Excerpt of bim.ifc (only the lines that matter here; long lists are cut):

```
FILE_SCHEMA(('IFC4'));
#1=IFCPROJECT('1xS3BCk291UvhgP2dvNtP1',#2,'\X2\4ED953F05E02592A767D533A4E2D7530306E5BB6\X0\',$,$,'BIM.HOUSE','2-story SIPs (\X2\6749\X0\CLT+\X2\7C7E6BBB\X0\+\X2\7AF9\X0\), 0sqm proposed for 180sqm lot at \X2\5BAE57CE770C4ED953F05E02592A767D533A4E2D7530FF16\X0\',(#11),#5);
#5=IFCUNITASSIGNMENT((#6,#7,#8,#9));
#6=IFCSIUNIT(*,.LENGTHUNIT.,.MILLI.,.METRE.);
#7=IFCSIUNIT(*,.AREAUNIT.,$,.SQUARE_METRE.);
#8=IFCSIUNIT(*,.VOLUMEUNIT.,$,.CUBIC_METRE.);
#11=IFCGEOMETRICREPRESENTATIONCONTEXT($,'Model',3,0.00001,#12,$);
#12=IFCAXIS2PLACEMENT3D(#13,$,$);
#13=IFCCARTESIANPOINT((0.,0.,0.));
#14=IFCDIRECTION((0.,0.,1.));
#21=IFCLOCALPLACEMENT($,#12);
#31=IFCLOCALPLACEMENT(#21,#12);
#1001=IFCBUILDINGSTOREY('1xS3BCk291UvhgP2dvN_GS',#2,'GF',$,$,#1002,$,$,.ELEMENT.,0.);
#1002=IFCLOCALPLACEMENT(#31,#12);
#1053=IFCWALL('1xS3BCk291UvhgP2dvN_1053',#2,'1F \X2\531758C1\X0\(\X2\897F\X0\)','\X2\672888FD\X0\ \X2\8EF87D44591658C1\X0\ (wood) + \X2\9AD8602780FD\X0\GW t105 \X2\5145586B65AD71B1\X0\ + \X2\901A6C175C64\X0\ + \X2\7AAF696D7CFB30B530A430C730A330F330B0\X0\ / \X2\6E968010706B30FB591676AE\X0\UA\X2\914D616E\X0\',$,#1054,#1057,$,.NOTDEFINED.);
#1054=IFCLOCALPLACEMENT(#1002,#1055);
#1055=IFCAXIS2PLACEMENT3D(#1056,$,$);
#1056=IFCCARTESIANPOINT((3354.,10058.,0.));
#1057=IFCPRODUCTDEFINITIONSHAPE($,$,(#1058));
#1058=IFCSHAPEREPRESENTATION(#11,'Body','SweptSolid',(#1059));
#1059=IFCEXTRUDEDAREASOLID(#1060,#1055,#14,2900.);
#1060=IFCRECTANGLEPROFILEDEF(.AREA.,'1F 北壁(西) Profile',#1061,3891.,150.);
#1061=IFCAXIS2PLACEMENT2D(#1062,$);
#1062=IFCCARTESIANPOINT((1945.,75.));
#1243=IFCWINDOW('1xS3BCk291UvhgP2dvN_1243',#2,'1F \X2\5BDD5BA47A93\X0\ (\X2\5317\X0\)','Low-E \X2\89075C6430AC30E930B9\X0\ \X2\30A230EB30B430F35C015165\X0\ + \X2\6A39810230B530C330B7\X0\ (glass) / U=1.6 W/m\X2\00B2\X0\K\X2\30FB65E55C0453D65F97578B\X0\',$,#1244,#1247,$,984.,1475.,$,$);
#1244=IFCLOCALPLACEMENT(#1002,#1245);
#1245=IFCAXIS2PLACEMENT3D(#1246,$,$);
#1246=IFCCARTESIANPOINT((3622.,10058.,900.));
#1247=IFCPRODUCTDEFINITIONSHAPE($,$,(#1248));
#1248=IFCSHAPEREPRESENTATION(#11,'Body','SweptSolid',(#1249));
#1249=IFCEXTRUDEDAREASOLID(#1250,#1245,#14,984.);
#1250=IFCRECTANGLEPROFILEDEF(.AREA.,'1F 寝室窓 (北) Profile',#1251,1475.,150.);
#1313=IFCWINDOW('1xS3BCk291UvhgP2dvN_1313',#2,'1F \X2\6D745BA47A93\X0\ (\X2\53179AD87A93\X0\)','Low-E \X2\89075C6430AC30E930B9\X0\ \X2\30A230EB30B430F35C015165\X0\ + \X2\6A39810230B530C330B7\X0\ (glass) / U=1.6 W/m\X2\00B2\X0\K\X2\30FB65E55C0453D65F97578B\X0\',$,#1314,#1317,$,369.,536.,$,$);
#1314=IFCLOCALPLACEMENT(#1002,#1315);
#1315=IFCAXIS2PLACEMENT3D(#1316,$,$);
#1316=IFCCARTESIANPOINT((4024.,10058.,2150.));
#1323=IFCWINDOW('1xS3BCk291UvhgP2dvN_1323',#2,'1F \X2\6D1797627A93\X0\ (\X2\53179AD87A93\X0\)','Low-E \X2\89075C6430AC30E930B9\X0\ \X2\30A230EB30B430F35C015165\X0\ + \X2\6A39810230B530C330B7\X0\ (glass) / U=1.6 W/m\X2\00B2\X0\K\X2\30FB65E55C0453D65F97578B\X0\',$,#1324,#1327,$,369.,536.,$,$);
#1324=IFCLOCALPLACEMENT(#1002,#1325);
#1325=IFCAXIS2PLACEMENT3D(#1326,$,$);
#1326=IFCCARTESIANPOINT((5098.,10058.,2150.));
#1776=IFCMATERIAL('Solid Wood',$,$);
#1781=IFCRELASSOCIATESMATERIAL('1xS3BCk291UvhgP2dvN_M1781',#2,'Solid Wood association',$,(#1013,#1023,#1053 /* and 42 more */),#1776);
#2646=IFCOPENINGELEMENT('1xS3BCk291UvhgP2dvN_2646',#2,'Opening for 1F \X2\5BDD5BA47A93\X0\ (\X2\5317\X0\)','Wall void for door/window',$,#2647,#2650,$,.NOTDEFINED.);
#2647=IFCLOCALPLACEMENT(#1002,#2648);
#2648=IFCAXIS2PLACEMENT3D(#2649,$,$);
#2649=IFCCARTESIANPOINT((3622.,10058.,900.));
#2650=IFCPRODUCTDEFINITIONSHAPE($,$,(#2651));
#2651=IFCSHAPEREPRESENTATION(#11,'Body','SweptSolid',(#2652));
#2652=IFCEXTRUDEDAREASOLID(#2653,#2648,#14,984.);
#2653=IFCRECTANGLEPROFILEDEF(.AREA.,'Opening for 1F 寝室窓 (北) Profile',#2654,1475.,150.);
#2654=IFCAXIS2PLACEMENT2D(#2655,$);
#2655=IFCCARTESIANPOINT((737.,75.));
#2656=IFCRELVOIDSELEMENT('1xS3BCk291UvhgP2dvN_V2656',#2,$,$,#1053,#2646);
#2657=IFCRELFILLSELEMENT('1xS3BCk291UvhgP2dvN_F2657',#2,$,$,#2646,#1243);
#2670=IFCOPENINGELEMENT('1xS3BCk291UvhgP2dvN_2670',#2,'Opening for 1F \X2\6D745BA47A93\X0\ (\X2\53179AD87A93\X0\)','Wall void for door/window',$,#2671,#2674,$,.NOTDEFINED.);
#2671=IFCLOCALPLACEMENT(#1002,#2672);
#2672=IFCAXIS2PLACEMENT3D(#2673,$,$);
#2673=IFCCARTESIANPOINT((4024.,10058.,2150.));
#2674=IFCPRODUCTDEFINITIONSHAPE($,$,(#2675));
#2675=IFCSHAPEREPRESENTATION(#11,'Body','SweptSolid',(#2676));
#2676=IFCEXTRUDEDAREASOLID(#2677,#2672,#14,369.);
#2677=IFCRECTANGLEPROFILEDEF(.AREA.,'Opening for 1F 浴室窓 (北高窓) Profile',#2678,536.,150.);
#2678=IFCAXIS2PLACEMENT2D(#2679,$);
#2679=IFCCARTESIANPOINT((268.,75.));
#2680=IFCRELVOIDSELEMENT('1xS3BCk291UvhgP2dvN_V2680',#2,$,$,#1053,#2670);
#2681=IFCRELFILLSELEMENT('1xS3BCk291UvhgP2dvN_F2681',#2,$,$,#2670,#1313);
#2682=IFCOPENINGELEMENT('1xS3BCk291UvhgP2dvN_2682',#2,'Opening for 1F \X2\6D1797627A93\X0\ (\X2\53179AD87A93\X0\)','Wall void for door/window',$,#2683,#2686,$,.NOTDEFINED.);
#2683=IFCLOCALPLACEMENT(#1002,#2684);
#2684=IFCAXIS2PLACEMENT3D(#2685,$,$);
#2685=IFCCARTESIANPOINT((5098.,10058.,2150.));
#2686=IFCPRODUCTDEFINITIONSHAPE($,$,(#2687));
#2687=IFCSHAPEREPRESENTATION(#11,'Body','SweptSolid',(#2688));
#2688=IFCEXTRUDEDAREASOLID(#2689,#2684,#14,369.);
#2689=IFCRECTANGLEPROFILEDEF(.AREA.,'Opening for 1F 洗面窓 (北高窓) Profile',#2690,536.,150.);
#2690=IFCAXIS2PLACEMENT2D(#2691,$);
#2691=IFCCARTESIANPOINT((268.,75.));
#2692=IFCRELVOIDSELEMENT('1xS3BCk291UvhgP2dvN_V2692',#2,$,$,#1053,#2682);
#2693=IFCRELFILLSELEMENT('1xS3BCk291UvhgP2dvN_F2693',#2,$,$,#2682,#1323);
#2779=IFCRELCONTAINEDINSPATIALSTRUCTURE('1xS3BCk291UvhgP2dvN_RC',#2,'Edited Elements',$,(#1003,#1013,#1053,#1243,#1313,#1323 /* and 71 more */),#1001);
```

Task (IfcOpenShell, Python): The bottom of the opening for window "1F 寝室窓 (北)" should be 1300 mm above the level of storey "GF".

```python
import numpy as np
import ifcopenshell
import ifcopenshell.api.geometry
import ifcopenshell.geom
import ifcopenshell.util.element
import ifcopenshell.util.placement
import ifcopenshell.util.shape
import ifcopenshell.util.unit

model = ifcopenshell.open("bim.ifc")
unit_scale = ifcopenshell.util.unit.calculate_unit_scale(model)

window = model.by_guid("1xS3BCk291UvhgP2dvN_1243")
opening = window.FillsVoids[0].RelatingOpeningElement
storey = ifcopenshell.util.element.get_container(window, ifc_class="IfcBuildingStorey")
level = ifcopenshell.util.placement.get_local_placement(storey.ObjectPlacement)[2, 3]

# The opening's origin need not be at the sill, so measure its lowest point.
shape = ifcopenshell.geom.create_shape(ifcopenshell.geom.settings(), opening)
bottom = ifcopenshell.util.shape.get_shape_bottom_elevation(shape, shape.geometry) / unit_scale
dz = level + 1.3 / unit_scale - bottom

shift = np.array([0.0, 0.0, dz])
# The window is not placed relative to its opening, so move both.
for product in (opening, window):
    matrix = ifcopenshell.util.placement.get_local_placement(product.ObjectPlacement)
    matrix[:3, 3] += shift
    ifcopenshell.api.geometry.edit_object_placement(model, product=product, matrix=matrix, is_si=False)

print(f"moved by {dz * unit_scale:+.3f} m")

model.write("bim_edited.ifc")
```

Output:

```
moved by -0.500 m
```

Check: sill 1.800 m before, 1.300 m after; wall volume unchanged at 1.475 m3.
